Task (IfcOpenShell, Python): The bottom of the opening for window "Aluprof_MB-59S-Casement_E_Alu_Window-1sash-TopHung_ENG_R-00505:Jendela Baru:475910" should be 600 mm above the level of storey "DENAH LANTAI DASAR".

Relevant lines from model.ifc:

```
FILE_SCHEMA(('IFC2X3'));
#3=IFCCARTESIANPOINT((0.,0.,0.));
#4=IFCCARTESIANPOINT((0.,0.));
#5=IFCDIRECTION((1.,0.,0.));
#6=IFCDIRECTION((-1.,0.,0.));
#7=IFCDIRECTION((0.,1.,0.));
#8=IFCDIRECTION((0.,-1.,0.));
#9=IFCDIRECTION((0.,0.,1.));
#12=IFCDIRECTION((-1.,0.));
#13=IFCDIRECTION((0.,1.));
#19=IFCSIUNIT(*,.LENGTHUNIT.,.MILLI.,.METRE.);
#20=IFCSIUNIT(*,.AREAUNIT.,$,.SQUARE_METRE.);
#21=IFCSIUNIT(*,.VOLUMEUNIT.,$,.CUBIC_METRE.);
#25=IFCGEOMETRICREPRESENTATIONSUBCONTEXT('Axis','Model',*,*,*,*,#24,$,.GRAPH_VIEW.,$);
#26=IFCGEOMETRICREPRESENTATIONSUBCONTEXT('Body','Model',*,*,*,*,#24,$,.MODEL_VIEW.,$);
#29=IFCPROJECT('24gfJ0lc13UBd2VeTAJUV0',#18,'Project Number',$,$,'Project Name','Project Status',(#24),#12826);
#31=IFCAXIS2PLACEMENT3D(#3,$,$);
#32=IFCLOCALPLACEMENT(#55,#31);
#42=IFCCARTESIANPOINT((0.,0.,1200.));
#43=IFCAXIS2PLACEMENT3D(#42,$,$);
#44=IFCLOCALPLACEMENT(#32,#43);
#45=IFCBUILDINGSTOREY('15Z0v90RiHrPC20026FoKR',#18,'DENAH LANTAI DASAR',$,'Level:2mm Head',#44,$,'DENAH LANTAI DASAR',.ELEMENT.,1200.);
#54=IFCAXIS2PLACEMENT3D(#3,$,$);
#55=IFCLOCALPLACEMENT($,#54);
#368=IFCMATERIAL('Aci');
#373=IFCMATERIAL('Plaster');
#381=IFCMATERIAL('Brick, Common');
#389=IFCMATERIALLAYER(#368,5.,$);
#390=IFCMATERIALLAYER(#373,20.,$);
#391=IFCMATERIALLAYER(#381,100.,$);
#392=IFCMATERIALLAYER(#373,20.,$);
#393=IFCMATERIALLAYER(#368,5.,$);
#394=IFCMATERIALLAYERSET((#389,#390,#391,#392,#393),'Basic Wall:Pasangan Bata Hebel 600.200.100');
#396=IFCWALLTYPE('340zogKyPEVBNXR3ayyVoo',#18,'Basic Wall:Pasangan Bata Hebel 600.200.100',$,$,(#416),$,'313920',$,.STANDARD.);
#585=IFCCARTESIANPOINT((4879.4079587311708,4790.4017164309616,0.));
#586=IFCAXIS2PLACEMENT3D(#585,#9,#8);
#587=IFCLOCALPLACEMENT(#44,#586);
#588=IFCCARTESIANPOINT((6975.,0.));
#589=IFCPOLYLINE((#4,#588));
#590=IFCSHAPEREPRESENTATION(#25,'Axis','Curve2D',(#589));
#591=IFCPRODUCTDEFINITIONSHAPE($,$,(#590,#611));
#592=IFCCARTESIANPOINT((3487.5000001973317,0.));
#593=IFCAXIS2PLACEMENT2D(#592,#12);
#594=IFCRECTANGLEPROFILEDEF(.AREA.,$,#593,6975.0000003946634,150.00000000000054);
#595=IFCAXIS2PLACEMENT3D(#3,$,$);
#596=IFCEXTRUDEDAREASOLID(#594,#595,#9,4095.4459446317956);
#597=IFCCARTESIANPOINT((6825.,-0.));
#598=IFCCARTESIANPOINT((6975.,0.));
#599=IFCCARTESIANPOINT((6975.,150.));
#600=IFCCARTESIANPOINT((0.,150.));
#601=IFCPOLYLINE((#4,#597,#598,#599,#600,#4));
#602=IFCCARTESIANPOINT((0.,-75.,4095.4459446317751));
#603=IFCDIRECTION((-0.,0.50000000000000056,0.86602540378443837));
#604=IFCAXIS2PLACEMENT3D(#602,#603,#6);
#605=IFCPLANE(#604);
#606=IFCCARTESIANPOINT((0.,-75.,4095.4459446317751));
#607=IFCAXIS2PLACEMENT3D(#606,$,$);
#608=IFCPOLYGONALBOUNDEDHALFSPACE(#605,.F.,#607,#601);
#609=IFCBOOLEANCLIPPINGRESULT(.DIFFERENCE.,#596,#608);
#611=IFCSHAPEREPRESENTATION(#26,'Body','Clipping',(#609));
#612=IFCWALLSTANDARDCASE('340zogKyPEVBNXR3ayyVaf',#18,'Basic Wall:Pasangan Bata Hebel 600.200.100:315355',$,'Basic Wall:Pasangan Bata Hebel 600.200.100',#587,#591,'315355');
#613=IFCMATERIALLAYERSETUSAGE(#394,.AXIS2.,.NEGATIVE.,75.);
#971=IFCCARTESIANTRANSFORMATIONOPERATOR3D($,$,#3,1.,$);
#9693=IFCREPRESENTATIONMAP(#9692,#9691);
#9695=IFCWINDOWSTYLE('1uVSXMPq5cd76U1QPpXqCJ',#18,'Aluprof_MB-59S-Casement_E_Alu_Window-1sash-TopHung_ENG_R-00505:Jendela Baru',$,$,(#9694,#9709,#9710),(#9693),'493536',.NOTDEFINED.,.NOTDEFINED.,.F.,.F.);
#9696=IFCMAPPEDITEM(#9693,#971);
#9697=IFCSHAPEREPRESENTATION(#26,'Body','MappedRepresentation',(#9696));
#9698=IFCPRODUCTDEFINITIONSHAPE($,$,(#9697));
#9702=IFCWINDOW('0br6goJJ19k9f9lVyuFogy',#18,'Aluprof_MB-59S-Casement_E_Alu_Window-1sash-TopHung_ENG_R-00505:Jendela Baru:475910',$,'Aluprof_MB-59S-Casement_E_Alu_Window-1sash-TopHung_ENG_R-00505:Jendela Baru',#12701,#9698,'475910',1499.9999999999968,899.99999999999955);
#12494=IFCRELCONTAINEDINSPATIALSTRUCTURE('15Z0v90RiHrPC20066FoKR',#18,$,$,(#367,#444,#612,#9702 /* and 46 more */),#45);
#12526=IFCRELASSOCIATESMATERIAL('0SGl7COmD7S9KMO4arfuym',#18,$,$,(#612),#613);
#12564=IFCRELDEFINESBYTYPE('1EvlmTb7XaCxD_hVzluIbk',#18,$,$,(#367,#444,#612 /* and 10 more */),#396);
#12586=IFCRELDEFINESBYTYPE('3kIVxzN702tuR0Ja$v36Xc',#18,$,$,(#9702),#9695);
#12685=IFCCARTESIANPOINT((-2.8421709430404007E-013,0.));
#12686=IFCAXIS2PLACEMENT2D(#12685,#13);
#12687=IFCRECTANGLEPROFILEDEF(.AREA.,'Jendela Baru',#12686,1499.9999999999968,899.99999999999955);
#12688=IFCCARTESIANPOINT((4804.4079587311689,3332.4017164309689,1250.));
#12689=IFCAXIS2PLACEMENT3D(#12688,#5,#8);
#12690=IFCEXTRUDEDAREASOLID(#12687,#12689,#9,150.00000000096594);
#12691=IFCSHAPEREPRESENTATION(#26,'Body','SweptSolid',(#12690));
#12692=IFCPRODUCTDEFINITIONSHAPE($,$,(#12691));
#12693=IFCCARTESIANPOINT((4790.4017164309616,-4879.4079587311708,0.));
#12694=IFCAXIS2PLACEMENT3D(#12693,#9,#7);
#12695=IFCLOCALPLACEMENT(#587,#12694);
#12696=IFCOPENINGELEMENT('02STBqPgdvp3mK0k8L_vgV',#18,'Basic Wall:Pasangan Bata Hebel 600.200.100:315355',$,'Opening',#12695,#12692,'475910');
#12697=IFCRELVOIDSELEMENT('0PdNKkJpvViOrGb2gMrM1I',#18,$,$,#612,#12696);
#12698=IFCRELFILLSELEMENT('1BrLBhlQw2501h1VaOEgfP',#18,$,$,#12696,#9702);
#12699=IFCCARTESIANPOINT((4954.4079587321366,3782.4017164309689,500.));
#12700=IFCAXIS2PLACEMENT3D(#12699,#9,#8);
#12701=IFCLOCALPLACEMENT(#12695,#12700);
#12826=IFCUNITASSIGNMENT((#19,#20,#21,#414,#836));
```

```python
import numpy as np
import ifcopenshell
import ifcopenshell.api.geometry
import ifcopenshell.geom
import ifcopenshell.util.element
import ifcopenshell.util.placement
import ifcopenshell.util.shape
import ifcopenshell.util.unit

model = ifcopenshell.open("model.ifc")
unit_scale = ifcopenshell.util.unit.calculate_unit_scale(model)

window = model.by_guid("0br6goJJ19k9f9lVyuFogy")
opening = window.FillsVoids[0].RelatingOpeningElement
storey = ifcopenshell.util.element.get_container(window, ifc_class="IfcBuildingStorey")
level = ifcopenshell.util.placement.get_local_placement(storey.ObjectPlacement)[2, 3]

# The opening's origin need not be at the sill, so measure its lowest point.
shape = ifcopenshell.geom.create_shape(ifcopenshell.geom.settings(), opening)
bottom = ifcopenshell.util.shape.get_shape_bottom_elevation(shape, shape.geometry) / unit_scale
dz = level + 0.6 / unit_scale - bottom

shift = np.array([0.0, 0.0, dz])
# The window is placed relative to its opening, so it follows when the opening moves.
matrix = ifcopenshell.util.placement.get_local_placement(opening.ObjectPlacement)
matrix[:3, 3] += shift
ifcopenshell.api.geometry.edit_object_placement(
    model, product=opening, matrix=matrix, is_si=False, should_transform_children=True
)

print(f"moved by {dz * unit_scale:+.3f} m")

model.write("model_v2.ifc")
```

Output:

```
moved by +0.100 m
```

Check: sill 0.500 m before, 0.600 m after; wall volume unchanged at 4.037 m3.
